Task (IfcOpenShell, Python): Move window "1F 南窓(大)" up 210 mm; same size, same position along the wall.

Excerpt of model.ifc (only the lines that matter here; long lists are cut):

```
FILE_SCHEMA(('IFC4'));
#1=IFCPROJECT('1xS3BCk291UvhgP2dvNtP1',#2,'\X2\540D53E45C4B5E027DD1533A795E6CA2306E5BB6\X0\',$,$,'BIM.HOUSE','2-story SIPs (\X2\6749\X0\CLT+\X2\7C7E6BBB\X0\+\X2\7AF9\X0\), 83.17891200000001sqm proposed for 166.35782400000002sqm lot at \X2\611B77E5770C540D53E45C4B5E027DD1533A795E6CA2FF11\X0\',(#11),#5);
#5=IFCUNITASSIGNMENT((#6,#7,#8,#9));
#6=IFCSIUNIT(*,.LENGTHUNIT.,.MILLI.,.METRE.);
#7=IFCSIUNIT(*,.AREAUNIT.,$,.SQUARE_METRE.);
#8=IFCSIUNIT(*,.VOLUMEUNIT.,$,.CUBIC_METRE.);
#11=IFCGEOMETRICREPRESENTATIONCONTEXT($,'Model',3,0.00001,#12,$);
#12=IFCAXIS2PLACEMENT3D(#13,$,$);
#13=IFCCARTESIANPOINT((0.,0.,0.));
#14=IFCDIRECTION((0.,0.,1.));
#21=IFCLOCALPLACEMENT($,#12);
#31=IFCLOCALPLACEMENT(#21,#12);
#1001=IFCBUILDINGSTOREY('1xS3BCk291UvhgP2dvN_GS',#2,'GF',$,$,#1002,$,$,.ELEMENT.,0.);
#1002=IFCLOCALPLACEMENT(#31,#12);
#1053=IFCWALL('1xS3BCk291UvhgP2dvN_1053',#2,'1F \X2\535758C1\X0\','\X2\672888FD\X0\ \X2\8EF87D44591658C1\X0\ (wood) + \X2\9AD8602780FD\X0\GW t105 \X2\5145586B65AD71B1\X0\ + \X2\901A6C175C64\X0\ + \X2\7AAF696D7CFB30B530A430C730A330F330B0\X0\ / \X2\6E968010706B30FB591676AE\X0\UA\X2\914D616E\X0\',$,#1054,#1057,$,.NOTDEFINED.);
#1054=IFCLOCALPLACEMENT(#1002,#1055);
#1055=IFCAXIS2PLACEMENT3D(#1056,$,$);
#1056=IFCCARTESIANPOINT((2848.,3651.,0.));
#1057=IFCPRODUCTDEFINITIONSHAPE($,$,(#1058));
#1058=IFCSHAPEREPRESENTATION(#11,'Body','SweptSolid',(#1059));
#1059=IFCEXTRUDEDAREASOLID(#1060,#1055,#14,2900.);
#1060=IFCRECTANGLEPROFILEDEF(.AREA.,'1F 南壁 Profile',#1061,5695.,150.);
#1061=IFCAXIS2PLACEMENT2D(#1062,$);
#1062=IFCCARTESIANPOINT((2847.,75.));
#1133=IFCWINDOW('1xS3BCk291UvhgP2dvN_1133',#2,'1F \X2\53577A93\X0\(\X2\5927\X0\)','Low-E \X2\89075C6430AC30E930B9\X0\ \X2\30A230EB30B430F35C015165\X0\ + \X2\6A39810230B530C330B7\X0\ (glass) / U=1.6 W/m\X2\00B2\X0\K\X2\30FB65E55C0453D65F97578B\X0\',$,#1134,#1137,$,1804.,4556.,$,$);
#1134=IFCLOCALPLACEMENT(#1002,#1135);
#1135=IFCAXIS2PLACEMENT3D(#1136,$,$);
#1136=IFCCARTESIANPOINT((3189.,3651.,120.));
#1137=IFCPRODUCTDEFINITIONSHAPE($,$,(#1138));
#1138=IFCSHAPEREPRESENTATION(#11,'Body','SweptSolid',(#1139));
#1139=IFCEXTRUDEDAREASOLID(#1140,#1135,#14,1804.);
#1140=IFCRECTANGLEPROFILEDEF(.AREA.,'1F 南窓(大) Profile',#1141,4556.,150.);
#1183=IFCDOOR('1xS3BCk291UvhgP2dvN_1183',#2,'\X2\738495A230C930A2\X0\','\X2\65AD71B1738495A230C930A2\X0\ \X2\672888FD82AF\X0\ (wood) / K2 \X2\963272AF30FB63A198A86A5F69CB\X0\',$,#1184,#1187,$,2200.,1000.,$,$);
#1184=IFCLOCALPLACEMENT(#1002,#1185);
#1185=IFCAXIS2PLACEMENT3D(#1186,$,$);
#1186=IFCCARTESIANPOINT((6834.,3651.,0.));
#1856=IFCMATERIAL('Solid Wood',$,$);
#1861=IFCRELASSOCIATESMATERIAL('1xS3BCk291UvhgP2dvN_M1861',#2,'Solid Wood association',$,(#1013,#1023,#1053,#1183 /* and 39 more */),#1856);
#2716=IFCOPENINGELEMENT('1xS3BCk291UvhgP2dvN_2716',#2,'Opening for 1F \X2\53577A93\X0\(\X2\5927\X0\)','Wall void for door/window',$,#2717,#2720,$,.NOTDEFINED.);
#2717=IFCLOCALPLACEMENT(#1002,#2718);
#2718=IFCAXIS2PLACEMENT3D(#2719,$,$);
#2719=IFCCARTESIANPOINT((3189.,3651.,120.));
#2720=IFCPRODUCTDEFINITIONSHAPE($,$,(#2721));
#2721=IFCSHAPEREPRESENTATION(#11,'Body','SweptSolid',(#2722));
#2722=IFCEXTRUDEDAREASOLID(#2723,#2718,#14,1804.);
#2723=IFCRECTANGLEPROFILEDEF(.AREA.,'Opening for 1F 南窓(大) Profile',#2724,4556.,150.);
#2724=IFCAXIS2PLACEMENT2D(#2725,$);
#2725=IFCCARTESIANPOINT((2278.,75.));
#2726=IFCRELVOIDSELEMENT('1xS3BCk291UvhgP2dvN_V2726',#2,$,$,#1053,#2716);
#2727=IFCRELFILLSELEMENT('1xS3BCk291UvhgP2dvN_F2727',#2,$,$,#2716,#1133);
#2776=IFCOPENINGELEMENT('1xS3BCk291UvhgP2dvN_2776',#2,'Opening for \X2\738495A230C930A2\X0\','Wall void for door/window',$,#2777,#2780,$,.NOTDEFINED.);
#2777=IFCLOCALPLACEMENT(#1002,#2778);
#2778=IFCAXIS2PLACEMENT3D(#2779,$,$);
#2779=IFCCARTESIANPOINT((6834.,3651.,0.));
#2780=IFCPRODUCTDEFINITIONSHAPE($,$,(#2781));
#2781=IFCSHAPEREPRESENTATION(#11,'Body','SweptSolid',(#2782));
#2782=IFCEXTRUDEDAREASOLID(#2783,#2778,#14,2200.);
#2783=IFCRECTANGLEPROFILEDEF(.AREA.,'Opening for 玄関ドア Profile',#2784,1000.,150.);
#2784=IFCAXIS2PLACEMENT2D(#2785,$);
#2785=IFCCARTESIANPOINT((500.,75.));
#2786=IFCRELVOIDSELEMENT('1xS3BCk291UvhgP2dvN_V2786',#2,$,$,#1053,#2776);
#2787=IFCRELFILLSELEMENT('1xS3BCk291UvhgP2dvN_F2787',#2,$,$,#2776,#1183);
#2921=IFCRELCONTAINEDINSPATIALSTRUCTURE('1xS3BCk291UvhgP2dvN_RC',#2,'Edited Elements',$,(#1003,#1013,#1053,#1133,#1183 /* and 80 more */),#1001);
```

```python
import numpy as np
import ifcopenshell
import ifcopenshell.api.geometry
import ifcopenshell.util.placement
import ifcopenshell.util.unit

model = ifcopenshell.open("model.ifc")
unit_scale = ifcopenshell.util.unit.calculate_unit_scale(model)

window = model.by_id(1133)
opening = window.FillsVoids[0].RelatingOpeningElement
dz = 0.21 / unit_scale

shift = np.array([0.0, 0.0, dz])
# The window is not placed relative to its opening, so move both.
for product in (opening, window):
    matrix = ifcopenshell.util.placement.get_local_placement(product.ObjectPlacement)
    matrix[:3, 3] += shift
    ifcopenshell.api.geometry.edit_object_placement(model, product=product, matrix=matrix, is_si=False)

print(f"moved by {dz * unit_scale:+.3f} m")

model.write("model_updated.ifc")
```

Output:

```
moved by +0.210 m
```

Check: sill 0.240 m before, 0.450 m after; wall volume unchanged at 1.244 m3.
